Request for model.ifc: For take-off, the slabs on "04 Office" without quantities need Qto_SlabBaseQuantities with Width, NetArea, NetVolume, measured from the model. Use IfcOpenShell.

First a look at what the model holds.

```python
import ifcopenshell
import ifcopenshell.util.element
import ifcopenshell.util.unit

model = ifcopenshell.open("model.ifc")
print(model.schema)
for unit_type in ("LENGTHUNIT", "AREAUNIT", "VOLUMEUNIT"):
    print(unit_type, ifcopenshell.util.unit.calculate_unit_scale(model, unit_type))
storey = next(s for s in model.by_type("IfcBuildingStorey") if s.Name == "04 Office")
slabs = [e for e in ifcopenshell.util.element.get_decomposition(storey) if e.is_a("IfcSlab")]
for e in sorted(slabs, key=lambda e: e.id()):
    print(e.id(), e.is_a(), e.Name, list(ifcopenshell.util.element.get_psets(e, qtos_only=True)), sep=" | ")
```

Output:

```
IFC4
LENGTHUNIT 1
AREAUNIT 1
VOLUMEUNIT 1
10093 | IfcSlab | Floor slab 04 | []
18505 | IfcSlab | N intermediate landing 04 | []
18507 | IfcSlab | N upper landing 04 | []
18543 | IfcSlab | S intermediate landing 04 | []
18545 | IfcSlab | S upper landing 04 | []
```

```python
import ifcopenshell
import ifcopenshell.api.pset
import ifcopenshell.geom
import ifcopenshell.util.element
import ifcopenshell.util.shape
import ifcopenshell.util.unit

model = ifcopenshell.open("model.ifc")
unit_scale = ifcopenshell.util.unit.calculate_unit_scale(model)
area_scale = ifcopenshell.util.unit.calculate_unit_scale(model, "AREAUNIT")
volume_scale = ifcopenshell.util.unit.calculate_unit_scale(model, "VOLUMEUNIT")
settings = ifcopenshell.geom.settings()

storey = next(s for s in model.by_type("IfcBuildingStorey") if s.Name == "04 Office")
slabs = [e for e in ifcopenshell.util.element.get_decomposition(storey) if e.is_a("IfcSlab")]

for e in sorted(slabs, key=lambda e: e.id()):
    if ifcopenshell.util.element.get_psets(e, qtos_only=True, should_inherit=False):
        continue
    # Geometry comes back in metres, in the element's own axes.
    shape = ifcopenshell.geom.create_shape(settings, e)
    values = {
        "Width": ifcopenshell.util.shape.get_z(shape.geometry) / unit_scale,
        "NetArea": ifcopenshell.util.shape.get_footprint_area(shape.geometry) / area_scale,
        "NetVolume": ifcopenshell.util.shape.get_volume(shape.geometry) / volume_scale,
    }
    qto = ifcopenshell.api.pset.add_qto(model, product=e, name="Qto_SlabBaseQuantities")
    ifcopenshell.api.pset.edit_qto(model, qto=qto, properties=values)
    print(e.id(), {k: round(v, 3) for k, v in values.items()})

model.write("model_v2.ifc")
```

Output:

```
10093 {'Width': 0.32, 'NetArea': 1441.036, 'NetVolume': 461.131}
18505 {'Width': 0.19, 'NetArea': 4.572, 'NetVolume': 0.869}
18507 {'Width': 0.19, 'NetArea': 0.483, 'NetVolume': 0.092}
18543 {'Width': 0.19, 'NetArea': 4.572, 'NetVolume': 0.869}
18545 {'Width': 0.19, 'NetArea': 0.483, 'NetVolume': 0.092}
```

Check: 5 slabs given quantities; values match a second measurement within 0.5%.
